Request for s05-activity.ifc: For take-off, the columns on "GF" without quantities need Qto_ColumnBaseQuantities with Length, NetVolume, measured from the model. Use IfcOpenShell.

First a look at what the model holds.

```python
import ifcopenshell
import ifcopenshell.util.element
import ifcopenshell.util.unit

model = ifcopenshell.open("s05-activity.ifc")
print(model.schema)
for unit_type in ("LENGTHUNIT", "AREAUNIT", "VOLUMEUNIT"):
    print(unit_type, ifcopenshell.util.unit.calculate_unit_scale(model, unit_type))
storey = next(s for s in model.by_type("IfcBuildingStorey") if s.Name == "GF")
columns = [e for e in ifcopenshell.util.element.get_decomposition(storey) if e.is_a("IfcColumn")]
for e in sorted(columns, key=lambda e: e.id()):
    print(e.id(), e.is_a(), e.Name, list(ifcopenshell.util.element.get_psets(e, qtos_only=True)), sep=" | ")
```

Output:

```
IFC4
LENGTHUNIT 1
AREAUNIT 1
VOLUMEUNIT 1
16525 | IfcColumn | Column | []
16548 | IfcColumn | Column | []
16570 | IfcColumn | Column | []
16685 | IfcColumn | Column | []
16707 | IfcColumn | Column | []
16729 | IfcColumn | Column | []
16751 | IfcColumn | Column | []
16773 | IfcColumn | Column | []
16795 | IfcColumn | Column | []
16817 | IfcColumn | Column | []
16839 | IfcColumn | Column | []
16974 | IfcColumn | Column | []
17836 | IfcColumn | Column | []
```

```python
import ifcopenshell
import ifcopenshell.api.pset
import ifcopenshell.geom
import ifcopenshell.util.element
import ifcopenshell.util.shape
import ifcopenshell.util.unit

model = ifcopenshell.open("s05-activity.ifc")
unit_scale = ifcopenshell.util.unit.calculate_unit_scale(model)
volume_scale = ifcopenshell.util.unit.calculate_unit_scale(model, "VOLUMEUNIT")
settings = ifcopenshell.geom.settings()

storey = next(s for s in model.by_type("IfcBuildingStorey") if s.Name == "GF")
columns = [e for e in ifcopenshell.util.element.get_decomposition(storey) if e.is_a("IfcColumn")]

for e in sorted(columns, key=lambda e: e.id()):
    if ifcopenshell.util.element.get_psets(e, qtos_only=True, should_inherit=False):
        continue
    # Geometry comes back in metres, in the element's own axes.
    shape = ifcopenshell.geom.create_shape(settings, e)
    values = {
        "Length": ifcopenshell.util.shape.get_z(shape.geometry) / unit_scale,
        "NetVolume": ifcopenshell.util.shape.get_volume(shape.geometry) / volume_scale,
    }
    qto = ifcopenshell.api.pset.add_qto(model, product=e, name="Qto_ColumnBaseQuantities")
    ifcopenshell.api.pset.edit_qto(model, qto=qto, properties=values)
    print(e.id(), {k: round(v, 3) for k, v in values.items()})

model.write("s05-activity-out.ifc")
```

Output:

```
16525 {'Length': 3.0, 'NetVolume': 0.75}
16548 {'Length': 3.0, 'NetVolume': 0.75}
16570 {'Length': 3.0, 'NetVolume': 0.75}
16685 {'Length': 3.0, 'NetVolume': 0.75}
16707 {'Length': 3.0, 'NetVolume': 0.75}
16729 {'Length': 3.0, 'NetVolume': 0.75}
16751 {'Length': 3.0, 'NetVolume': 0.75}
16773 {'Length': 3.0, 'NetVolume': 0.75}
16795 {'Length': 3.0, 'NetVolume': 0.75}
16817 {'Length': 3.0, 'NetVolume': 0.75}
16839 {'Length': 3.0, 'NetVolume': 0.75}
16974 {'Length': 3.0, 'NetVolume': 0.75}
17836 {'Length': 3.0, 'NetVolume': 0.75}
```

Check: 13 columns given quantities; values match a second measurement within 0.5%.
